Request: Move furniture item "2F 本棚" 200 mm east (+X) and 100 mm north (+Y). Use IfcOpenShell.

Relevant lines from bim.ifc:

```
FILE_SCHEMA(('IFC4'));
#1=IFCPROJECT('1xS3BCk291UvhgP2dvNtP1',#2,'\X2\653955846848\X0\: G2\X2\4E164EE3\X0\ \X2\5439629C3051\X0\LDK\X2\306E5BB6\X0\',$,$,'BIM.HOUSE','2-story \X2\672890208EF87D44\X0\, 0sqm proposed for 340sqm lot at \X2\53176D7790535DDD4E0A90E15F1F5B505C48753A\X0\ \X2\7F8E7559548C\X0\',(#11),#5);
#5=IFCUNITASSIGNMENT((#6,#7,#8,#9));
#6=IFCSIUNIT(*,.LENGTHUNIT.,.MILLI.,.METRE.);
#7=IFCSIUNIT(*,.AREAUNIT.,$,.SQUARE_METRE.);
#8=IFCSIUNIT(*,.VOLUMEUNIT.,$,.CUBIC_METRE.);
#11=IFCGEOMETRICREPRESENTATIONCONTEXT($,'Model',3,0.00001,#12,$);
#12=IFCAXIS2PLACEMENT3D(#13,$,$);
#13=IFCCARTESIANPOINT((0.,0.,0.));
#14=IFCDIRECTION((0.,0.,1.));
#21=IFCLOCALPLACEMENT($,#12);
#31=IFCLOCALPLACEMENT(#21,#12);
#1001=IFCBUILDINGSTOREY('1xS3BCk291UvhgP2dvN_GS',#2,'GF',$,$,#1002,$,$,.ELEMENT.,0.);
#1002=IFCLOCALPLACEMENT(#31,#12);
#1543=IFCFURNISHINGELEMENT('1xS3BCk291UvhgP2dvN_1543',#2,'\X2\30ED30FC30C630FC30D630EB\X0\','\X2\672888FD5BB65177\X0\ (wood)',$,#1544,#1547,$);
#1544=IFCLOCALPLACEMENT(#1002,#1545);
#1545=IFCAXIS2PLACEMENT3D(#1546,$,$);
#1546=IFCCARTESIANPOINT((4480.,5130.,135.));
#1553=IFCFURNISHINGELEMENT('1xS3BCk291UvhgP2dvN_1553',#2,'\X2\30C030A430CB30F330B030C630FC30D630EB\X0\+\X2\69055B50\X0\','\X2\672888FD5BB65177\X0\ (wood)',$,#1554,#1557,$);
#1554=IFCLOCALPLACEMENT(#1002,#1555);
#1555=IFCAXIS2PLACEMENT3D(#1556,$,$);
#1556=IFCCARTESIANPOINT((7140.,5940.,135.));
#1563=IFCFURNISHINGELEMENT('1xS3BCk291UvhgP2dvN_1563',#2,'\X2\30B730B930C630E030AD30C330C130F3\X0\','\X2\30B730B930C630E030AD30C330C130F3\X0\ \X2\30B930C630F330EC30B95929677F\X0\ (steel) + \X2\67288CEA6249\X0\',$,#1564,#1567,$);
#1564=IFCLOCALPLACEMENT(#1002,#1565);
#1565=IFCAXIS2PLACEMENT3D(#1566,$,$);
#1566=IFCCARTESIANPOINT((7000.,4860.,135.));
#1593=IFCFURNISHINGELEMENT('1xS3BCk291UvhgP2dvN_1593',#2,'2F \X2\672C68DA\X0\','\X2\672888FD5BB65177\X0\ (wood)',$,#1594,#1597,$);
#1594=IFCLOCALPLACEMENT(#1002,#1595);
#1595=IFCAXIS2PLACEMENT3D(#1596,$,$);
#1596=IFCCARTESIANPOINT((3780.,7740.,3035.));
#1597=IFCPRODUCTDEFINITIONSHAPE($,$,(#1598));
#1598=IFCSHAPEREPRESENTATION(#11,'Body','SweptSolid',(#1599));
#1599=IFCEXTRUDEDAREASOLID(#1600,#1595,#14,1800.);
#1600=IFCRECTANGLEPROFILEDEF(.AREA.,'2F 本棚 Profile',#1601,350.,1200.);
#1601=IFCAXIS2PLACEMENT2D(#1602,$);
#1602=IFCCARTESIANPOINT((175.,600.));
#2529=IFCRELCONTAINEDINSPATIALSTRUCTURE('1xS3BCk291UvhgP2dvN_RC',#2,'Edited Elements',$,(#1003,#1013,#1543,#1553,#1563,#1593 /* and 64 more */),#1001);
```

```python
import ifcopenshell
import ifcopenshell.api.geometry
import ifcopenshell.util.placement
import ifcopenshell.util.unit

model = ifcopenshell.open("bim.ifc")
unit_scale = ifcopenshell.util.unit.calculate_unit_scale(model)

item = model.by_guid("1xS3BCk291UvhgP2dvN_1593")
matrix = ifcopenshell.util.placement.get_local_placement(item.ObjectPlacement)
matrix[0, 3] += 0.2 / unit_scale
matrix[1, 3] += 0.1 / unit_scale
ifcopenshell.api.geometry.edit_object_placement(model, product=item, matrix=matrix, is_si=False)

print(ifcopenshell.util.placement.get_local_placement(item.ObjectPlacement).round(3) + 0.0)

model.write("bim_rev.ifc")
```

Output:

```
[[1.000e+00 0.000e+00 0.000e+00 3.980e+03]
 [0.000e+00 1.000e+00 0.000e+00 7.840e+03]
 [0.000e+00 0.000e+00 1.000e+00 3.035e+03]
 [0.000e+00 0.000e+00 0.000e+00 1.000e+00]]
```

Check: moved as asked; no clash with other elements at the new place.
